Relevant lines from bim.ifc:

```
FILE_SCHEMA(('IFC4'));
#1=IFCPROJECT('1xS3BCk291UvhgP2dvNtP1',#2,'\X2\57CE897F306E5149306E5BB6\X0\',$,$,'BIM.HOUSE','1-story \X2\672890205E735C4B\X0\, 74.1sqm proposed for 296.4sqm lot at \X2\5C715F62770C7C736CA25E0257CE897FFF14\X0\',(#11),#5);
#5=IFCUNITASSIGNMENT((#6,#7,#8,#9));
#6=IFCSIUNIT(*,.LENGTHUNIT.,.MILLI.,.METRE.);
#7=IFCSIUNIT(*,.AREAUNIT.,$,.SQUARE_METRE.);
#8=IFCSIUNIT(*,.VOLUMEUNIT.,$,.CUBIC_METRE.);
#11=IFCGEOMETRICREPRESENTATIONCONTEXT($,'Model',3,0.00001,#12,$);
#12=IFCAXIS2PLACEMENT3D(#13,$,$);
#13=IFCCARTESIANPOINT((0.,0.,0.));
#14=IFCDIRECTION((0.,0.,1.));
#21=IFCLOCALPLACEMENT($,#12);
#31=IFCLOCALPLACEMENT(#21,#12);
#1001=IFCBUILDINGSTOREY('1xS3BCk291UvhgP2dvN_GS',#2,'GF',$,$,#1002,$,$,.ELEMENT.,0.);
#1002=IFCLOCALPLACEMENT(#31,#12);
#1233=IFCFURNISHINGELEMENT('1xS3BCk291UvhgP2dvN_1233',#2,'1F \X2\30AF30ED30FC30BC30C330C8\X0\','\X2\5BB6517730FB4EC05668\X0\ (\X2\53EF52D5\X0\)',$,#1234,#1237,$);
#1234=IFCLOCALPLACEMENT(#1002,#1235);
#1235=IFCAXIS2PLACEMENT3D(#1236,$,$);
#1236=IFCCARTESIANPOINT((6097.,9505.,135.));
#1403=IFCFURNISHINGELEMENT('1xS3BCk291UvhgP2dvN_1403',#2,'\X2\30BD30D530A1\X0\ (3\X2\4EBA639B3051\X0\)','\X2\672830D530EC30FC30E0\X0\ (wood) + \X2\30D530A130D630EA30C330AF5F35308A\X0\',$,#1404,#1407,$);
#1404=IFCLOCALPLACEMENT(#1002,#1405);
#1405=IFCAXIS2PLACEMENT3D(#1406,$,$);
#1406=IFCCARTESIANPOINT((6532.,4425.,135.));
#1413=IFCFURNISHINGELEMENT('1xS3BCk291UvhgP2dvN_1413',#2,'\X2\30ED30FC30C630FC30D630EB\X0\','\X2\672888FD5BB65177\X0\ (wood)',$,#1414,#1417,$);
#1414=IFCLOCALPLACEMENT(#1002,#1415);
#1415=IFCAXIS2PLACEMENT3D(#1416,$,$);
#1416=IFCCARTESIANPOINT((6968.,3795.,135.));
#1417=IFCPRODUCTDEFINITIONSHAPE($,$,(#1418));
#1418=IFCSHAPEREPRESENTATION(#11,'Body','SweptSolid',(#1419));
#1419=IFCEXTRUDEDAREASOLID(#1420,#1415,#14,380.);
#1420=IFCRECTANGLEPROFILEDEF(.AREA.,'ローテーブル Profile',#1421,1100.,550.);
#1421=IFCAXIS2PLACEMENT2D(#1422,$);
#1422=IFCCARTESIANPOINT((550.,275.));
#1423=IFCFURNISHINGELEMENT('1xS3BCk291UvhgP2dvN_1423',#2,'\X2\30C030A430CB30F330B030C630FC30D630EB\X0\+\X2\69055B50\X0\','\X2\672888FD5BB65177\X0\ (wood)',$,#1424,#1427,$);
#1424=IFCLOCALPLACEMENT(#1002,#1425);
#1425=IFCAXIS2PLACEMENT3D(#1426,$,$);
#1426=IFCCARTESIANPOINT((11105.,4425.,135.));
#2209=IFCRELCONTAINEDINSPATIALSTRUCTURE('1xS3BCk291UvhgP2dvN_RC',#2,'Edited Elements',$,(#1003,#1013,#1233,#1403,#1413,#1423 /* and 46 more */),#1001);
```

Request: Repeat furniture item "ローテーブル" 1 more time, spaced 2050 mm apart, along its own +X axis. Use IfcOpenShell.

```python
import ifcopenshell
import ifcopenshell.api.geometry
import ifcopenshell.api.root
import ifcopenshell.util.element
import ifcopenshell.util.placement

model = ifcopenshell.open("bim.ifc")


def reuse_history(source, copy):
    """copy_class also copies each property set's owner history, people and application; keep the originals."""
    for rel in copy.IsDefinedBy:
        if rel.is_a("IfcRelDefinesByProperties") and (history := rel.RelatingPropertyDefinition.OwnerHistory):
            rel.RelatingPropertyDefinition.OwnerHistory = source.OwnerHistory
            ifcopenshell.util.element.remove_deep2(model, history)


source = model.by_guid("1xS3BCk291UvhgP2dvN_1413")
base = ifcopenshell.util.placement.get_local_placement(source.ObjectPlacement)
step = base[:3, 0] * 2050.0

for i in range(1, 2):
    copy = ifcopenshell.api.root.copy_class(model, product=source)
    copy.Representation = ifcopenshell.util.element.copy_deep(
        model, source.Representation, exclude=["IfcGeometricRepresentationContext", "IfcRepresentationMap"]
    )
    reuse_history(source, copy)
    matrix = base.copy()
    matrix[:3, 3] += i * step
    print("added at", matrix[:3, 3].round(3) + 0.0)
    ifcopenshell.api.geometry.edit_object_placement(model, product=copy, matrix=matrix, is_si=False)

model.write("bim_rev.ifc")
```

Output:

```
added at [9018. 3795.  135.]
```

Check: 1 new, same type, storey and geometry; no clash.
